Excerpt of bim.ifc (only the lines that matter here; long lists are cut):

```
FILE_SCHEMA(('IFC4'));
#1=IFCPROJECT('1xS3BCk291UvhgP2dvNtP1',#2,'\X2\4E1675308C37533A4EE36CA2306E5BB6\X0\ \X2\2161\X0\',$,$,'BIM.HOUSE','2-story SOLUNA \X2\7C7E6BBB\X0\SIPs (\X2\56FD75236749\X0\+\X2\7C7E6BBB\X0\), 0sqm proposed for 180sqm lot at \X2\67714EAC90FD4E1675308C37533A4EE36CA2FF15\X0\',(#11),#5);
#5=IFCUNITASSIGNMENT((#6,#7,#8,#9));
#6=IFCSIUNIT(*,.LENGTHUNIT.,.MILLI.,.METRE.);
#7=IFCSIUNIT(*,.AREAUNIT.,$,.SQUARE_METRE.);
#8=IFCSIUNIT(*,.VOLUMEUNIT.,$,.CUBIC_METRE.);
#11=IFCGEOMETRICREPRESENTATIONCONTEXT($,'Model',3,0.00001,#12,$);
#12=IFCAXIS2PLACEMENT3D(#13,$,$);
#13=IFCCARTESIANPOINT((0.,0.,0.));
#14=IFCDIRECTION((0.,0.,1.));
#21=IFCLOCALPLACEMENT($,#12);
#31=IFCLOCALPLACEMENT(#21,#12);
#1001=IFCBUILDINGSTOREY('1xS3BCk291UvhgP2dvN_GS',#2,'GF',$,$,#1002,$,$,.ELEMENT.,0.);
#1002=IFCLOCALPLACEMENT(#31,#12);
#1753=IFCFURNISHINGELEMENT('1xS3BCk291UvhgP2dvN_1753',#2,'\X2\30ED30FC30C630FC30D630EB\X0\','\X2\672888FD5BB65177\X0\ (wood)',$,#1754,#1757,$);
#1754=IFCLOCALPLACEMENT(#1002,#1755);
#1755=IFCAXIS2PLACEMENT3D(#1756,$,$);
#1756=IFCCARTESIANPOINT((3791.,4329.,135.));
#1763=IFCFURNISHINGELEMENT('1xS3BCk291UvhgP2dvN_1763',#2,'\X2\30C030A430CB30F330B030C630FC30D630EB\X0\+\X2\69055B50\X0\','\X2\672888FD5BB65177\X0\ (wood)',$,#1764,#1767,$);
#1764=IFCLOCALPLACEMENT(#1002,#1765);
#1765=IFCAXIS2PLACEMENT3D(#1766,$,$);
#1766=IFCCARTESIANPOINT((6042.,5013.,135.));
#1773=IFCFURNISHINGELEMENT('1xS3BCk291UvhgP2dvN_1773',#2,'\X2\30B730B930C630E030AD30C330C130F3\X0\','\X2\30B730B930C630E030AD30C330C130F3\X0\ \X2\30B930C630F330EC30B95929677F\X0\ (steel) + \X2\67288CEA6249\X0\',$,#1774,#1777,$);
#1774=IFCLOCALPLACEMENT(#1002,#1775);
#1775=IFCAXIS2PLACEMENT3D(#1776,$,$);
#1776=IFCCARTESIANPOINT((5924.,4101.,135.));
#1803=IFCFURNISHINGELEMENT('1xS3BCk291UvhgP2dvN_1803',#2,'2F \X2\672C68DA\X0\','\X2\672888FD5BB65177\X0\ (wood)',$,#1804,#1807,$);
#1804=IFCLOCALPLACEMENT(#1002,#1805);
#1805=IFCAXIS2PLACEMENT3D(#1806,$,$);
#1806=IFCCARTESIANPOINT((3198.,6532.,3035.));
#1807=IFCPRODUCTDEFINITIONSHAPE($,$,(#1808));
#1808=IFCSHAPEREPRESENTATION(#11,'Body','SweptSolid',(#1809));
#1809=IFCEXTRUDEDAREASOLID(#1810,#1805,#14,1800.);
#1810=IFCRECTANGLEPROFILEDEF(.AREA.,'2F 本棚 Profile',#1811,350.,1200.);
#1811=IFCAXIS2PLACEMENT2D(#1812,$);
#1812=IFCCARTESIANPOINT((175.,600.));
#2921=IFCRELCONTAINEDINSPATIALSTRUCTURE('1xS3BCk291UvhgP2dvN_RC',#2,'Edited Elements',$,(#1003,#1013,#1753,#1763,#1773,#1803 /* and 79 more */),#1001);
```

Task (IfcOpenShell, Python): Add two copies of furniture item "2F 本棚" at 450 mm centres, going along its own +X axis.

```python
import ifcopenshell
import ifcopenshell.api.geometry
import ifcopenshell.api.root
import ifcopenshell.util.element
import ifcopenshell.util.placement

model = ifcopenshell.open("bim.ifc")


def reuse_history(source, copy):
    """copy_class also copies each property set's owner history, people and application; keep the originals."""
    for rel in copy.IsDefinedBy:
        if rel.is_a("IfcRelDefinesByProperties") and (history := rel.RelatingPropertyDefinition.OwnerHistory):
            rel.RelatingPropertyDefinition.OwnerHistory = source.OwnerHistory
            ifcopenshell.util.element.remove_deep2(model, history)


source = model.by_guid("1xS3BCk291UvhgP2dvN_1803")
base = ifcopenshell.util.placement.get_local_placement(source.ObjectPlacement)
step = base[:3, 0] * 450.0

for i in range(1, 3):
    copy = ifcopenshell.api.root.copy_class(model, product=source)
    copy.Representation = ifcopenshell.util.element.copy_deep(
        model, source.Representation, exclude=["IfcGeometricRepresentationContext", "IfcRepresentationMap"]
    )
    reuse_history(source, copy)
    matrix = base.copy()
    matrix[:3, 3] += i * step
    print("added at", matrix[:3, 3].round(3) + 0.0)
    ifcopenshell.api.geometry.edit_object_placement(model, product=copy, matrix=matrix, is_si=False)

model.write("bim_rev.ifc")
```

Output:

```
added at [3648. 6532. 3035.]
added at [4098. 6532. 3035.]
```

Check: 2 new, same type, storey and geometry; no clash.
